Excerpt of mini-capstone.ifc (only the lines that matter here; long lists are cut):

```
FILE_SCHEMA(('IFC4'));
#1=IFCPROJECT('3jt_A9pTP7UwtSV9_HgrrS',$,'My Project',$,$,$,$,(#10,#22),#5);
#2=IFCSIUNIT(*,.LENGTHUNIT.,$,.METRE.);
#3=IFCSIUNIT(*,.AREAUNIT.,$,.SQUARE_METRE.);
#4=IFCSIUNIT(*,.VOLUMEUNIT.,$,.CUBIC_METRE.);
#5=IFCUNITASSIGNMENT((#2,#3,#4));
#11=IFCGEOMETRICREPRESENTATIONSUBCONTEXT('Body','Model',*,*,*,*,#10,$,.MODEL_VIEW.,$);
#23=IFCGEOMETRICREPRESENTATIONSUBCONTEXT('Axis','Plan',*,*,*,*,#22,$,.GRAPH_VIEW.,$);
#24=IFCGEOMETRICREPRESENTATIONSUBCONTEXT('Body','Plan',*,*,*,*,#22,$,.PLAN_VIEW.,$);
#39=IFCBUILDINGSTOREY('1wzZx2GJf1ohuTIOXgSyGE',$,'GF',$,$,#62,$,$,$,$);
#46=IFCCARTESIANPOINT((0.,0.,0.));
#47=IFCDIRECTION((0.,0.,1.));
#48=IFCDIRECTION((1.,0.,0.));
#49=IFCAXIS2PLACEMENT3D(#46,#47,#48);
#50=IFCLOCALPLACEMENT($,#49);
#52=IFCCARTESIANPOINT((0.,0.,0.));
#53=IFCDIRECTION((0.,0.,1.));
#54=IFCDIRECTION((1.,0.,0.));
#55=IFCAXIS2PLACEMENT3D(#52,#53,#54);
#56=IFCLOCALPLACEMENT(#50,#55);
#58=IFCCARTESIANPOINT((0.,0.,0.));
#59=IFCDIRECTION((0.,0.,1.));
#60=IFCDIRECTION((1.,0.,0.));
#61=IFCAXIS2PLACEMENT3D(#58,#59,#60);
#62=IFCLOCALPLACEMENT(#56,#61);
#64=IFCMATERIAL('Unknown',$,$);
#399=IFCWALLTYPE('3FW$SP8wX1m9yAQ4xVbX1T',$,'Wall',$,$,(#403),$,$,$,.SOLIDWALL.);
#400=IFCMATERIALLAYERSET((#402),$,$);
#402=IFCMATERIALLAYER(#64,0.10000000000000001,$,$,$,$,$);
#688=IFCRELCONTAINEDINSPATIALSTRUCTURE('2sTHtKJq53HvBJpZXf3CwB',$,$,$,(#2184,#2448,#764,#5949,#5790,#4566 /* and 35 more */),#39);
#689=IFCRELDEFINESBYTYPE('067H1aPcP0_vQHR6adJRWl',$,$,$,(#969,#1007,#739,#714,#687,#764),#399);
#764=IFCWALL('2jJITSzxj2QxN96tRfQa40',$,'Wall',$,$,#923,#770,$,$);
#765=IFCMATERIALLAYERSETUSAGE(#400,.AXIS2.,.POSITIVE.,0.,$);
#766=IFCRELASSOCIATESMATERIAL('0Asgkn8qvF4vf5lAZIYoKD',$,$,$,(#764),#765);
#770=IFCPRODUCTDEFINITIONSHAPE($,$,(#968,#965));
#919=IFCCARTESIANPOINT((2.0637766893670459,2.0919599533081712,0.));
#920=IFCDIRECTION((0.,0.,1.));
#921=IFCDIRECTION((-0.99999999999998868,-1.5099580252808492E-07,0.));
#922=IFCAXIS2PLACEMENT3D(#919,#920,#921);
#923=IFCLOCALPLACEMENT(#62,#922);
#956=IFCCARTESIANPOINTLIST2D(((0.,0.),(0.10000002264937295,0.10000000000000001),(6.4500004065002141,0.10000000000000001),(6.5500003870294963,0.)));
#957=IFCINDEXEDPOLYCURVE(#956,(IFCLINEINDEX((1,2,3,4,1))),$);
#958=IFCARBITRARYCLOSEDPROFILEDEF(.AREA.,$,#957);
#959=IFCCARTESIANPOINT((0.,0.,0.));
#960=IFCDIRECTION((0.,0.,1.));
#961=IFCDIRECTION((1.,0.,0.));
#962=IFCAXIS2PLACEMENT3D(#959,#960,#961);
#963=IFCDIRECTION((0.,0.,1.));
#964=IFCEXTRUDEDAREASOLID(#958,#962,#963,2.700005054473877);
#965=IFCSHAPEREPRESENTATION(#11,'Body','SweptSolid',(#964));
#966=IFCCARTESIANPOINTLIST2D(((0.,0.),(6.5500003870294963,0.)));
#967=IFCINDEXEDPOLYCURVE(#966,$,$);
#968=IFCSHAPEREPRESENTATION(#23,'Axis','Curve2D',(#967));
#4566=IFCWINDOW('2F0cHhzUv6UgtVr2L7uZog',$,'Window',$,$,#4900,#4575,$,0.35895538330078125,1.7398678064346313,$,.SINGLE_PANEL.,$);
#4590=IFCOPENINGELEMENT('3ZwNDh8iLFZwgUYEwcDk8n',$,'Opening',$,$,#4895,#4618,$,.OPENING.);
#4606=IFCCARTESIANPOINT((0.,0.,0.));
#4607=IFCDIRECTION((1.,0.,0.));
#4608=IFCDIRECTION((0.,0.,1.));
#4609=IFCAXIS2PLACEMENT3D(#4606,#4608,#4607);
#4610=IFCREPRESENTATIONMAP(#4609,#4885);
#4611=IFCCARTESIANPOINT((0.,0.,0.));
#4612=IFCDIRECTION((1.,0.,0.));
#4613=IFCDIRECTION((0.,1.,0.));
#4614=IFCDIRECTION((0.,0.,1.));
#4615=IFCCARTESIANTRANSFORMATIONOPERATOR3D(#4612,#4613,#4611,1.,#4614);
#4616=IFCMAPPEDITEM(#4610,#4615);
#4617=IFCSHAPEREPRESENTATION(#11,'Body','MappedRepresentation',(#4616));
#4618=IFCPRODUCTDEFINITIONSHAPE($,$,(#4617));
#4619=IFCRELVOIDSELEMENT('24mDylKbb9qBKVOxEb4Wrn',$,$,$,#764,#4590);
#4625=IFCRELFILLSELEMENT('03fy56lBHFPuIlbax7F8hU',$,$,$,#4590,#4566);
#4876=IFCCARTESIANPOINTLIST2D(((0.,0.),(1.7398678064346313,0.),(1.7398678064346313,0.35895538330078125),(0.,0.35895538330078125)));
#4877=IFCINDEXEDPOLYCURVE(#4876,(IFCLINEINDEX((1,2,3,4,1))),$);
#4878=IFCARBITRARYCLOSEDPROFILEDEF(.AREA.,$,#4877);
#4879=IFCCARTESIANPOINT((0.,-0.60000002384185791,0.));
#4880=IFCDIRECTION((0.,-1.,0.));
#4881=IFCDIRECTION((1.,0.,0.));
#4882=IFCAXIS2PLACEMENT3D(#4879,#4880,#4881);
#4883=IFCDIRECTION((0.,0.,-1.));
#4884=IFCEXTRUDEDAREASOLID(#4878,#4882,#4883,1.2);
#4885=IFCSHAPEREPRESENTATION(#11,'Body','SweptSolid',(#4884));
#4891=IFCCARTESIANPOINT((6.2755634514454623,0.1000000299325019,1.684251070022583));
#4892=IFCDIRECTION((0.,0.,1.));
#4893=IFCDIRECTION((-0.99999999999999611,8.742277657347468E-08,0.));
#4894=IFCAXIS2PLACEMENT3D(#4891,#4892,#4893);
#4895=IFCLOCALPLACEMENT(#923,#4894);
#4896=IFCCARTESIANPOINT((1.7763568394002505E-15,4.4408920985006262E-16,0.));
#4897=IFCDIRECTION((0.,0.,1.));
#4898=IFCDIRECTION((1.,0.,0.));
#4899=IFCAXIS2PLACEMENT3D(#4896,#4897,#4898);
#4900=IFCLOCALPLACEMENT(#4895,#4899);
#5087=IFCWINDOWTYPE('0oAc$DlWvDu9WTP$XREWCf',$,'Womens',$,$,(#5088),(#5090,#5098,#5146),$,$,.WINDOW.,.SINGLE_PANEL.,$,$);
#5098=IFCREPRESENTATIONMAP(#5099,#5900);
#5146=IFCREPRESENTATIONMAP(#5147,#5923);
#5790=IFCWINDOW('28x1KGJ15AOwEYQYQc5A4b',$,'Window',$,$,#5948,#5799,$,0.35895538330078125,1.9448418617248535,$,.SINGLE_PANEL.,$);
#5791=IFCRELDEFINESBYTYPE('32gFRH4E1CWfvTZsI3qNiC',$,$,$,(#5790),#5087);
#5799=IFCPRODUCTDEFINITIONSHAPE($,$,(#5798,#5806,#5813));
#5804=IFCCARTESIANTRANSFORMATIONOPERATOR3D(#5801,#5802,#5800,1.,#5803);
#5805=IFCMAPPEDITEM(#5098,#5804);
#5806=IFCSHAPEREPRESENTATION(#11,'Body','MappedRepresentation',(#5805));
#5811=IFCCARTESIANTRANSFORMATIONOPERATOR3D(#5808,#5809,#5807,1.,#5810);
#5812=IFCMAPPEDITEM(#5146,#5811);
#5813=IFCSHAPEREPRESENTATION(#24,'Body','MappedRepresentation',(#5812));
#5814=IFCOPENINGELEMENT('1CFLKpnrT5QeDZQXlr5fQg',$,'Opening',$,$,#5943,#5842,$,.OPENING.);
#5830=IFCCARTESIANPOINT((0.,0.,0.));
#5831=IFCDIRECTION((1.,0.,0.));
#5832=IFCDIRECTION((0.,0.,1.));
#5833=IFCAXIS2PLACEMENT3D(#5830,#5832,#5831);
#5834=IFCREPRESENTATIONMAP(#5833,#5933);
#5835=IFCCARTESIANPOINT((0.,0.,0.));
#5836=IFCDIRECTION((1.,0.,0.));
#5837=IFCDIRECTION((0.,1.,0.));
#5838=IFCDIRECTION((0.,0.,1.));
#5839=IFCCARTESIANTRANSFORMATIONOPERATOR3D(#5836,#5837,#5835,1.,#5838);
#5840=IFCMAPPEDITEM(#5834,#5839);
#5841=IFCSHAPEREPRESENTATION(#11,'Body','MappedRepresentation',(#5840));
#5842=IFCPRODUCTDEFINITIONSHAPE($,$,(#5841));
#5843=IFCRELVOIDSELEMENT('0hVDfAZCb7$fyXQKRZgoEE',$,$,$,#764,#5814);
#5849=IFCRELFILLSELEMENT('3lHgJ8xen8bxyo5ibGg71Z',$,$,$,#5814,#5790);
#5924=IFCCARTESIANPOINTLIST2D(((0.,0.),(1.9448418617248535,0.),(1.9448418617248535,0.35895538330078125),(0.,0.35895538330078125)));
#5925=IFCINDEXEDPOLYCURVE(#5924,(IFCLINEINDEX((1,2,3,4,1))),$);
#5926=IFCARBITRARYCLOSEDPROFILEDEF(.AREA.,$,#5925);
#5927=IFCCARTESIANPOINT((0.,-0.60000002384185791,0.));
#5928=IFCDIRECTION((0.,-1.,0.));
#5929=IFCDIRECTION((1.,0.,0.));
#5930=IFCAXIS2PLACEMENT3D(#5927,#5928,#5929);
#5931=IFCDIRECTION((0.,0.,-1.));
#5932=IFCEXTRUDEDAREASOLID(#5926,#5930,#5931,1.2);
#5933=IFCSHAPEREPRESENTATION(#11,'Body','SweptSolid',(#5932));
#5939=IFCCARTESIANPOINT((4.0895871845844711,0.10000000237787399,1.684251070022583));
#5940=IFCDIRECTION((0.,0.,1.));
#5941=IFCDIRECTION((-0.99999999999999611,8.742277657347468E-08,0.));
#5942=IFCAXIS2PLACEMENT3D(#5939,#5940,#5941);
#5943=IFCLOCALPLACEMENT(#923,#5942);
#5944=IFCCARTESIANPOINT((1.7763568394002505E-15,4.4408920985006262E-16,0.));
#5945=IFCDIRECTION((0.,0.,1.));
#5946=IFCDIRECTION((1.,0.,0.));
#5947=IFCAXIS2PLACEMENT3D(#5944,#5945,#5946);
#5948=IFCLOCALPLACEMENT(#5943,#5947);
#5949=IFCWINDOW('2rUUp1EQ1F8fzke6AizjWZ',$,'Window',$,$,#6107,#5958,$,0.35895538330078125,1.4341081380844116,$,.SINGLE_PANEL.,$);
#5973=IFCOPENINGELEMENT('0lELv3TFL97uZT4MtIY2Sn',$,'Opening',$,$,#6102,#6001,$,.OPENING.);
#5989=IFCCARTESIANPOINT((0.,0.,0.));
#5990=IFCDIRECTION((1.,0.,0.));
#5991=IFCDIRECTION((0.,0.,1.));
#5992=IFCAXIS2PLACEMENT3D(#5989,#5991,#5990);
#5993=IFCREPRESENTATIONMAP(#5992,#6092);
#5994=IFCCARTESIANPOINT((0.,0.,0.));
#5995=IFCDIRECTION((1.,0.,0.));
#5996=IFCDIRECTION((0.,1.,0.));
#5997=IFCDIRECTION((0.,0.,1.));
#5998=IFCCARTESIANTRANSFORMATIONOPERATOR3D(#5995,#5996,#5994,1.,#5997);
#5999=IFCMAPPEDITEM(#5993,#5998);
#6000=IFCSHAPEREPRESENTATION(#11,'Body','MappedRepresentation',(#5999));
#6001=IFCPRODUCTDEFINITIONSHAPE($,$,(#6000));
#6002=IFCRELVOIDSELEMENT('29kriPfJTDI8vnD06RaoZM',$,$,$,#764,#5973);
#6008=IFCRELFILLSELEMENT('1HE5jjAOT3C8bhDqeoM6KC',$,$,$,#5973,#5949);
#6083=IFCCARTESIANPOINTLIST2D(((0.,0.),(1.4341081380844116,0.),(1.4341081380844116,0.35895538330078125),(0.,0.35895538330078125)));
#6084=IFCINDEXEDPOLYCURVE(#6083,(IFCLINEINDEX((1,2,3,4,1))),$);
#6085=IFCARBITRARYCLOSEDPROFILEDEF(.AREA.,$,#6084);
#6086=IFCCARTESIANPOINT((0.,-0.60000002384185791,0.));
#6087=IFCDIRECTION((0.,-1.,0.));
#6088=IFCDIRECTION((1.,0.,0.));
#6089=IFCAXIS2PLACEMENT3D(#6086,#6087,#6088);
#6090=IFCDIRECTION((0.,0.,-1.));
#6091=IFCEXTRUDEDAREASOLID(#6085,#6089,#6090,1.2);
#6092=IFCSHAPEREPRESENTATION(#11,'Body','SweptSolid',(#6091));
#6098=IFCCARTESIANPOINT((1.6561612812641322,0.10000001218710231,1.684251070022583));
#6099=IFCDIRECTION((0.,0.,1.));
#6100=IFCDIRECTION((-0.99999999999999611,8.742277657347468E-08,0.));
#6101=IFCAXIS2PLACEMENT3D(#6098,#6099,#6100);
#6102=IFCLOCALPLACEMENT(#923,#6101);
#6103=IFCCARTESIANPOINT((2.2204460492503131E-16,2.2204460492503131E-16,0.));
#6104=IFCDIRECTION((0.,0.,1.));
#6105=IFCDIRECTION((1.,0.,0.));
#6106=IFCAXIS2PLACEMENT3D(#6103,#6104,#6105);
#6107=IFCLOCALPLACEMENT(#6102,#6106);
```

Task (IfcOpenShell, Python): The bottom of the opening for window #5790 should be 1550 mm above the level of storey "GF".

```python
import numpy as np
import ifcopenshell
import ifcopenshell.api.geometry
import ifcopenshell.geom
import ifcopenshell.util.element
import ifcopenshell.util.placement
import ifcopenshell.util.shape
import ifcopenshell.util.unit

model = ifcopenshell.open("mini-capstone.ifc")
unit_scale = ifcopenshell.util.unit.calculate_unit_scale(model)

window = model.by_guid("28x1KGJ15AOwEYQYQc5A4b")
opening = window.FillsVoids[0].RelatingOpeningElement
storey = ifcopenshell.util.element.get_container(window, ifc_class="IfcBuildingStorey")
level = ifcopenshell.util.placement.get_local_placement(storey.ObjectPlacement)[2, 3]

# The opening's origin need not be at the sill, so measure its lowest point.
shape = ifcopenshell.geom.create_shape(ifcopenshell.geom.settings(), opening)
bottom = ifcopenshell.util.shape.get_shape_bottom_elevation(shape, shape.geometry) / unit_scale
dz = level + 1.55 - bottom

shift = np.array([0.0, 0.0, dz])
# The window is placed relative to its opening, so it follows when the opening moves.
matrix = ifcopenshell.util.placement.get_local_placement(opening.ObjectPlacement)
matrix[:3, 3] += shift
ifcopenshell.api.geometry.edit_object_placement(
    model, product=opening, matrix=matrix, is_si=False, should_transform_children=True
)

print(f"moved by {dz * unit_scale:+.3f} m")

model.write("mini-capstone_rev.ifc")
```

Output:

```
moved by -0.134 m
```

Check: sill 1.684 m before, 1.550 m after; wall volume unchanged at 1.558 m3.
